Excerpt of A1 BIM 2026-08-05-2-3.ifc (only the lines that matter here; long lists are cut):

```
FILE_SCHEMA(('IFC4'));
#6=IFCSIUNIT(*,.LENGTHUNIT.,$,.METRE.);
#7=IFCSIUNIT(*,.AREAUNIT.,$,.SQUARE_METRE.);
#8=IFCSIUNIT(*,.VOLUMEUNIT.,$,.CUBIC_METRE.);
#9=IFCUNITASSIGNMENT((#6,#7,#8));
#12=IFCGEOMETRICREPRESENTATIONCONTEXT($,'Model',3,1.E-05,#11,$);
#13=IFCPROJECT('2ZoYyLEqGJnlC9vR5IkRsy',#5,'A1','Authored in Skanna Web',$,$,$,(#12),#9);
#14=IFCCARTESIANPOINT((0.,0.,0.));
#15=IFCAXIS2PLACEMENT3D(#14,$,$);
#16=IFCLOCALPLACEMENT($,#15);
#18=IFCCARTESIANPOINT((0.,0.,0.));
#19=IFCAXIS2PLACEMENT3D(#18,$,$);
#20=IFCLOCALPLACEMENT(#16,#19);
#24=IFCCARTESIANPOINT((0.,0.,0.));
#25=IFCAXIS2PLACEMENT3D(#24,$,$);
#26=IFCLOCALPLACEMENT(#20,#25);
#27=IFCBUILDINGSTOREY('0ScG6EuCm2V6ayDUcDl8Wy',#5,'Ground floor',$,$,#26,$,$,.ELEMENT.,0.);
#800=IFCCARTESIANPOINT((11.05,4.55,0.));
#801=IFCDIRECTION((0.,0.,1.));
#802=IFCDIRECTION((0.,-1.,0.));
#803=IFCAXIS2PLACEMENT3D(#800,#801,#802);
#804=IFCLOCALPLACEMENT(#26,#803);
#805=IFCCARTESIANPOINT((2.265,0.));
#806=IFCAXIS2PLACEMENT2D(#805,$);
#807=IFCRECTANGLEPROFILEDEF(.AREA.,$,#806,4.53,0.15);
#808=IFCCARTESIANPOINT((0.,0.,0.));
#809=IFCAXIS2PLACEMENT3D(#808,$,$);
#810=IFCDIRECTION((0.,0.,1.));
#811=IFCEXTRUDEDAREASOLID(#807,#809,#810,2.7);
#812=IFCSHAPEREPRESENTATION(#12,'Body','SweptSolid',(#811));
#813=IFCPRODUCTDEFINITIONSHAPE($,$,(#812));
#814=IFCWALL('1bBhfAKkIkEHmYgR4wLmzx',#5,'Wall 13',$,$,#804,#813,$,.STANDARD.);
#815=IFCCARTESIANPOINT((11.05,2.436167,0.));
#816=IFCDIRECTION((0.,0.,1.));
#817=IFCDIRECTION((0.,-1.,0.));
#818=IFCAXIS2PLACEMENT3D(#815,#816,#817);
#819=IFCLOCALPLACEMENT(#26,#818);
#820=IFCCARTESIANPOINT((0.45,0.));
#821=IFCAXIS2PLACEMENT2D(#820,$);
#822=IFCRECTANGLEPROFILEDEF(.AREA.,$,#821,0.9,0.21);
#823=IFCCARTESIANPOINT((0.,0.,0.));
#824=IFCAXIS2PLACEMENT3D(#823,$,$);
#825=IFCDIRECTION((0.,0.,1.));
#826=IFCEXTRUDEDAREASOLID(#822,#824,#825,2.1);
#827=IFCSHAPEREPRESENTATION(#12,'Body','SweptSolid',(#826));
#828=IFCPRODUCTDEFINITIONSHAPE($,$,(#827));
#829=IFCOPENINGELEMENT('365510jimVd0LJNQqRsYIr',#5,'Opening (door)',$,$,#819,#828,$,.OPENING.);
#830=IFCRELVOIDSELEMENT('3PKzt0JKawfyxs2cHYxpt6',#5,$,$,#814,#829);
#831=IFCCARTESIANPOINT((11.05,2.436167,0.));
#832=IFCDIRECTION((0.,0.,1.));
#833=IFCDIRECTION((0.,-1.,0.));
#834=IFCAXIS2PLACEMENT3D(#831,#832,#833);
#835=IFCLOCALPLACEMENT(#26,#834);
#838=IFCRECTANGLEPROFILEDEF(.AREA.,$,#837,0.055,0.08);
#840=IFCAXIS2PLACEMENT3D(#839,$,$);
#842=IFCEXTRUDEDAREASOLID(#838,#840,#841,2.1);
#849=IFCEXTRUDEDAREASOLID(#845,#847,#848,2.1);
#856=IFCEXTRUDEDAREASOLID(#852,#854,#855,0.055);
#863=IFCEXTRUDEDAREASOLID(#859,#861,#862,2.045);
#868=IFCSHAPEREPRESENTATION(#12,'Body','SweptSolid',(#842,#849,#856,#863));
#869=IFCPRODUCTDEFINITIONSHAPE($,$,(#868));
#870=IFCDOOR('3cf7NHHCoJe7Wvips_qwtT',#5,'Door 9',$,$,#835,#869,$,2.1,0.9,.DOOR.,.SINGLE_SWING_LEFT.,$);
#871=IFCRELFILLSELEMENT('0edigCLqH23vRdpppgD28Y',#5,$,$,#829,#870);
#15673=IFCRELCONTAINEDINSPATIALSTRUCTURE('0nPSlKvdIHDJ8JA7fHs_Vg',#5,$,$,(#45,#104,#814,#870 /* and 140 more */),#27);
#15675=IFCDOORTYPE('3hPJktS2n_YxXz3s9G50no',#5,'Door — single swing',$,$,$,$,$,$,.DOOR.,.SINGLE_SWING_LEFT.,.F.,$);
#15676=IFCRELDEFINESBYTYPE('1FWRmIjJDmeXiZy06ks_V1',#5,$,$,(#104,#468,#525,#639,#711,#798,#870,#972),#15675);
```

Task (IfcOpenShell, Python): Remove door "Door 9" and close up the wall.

```python
import ifcopenshell
import ifcopenshell.api.feature
import ifcopenshell.api.root
import ifcopenshell.geom
import ifcopenshell.util.shape

model = ifcopenshell.open("A1 BIM 2026-08-05-2-3.ifc")
settings = ifcopenshell.geom.settings()


def volume(element):
    """Net volume in cubic metres, openings subtracted."""
    shape = ifcopenshell.geom.create_shape(settings, element)
    return ifcopenshell.util.shape.get_volume(shape.geometry)


door = model.by_guid("3cf7NHHCoJe7Wvips_qwtT")
opening = door.FillsVoids[0].RelatingOpeningElement
wall = opening.VoidsElements[0].RelatingBuildingElement
before = volume(wall)

ifcopenshell.api.root.remove_product(model, product=door)
ifcopenshell.api.feature.remove_feature(model, feature=opening)

after = volume(wall)

print(f"wall volume {before:.3f} -> {after:.3f} m3")

model.write("A1 BIM 2026-08-05-2-3-out.ifc")
```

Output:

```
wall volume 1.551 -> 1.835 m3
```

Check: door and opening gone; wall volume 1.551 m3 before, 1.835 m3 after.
